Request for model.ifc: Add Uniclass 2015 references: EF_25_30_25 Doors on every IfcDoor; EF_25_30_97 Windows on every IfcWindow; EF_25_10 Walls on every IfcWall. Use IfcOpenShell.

First a look at what the model holds.

```python
import ifcopenshell

model = ifcopenshell.open("model.ifc")
print(model.schema)
print("classifications:", [c.Name for c in model.by_type("IfcClassification")])
for ifc_class in ("IfcDoor", "IfcRoof", "IfcStair", "IfcWall", "IfcWindow"):
    print(ifc_class, len(model.by_type(ifc_class)))
```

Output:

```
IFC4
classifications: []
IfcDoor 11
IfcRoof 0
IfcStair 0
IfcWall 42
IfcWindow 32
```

```python
import ifcopenshell
import ifcopenshell.api.classification

model = ifcopenshell.open("model.ifc")

system = ifcopenshell.api.classification.add_classification(model, classification="Uniclass 2015")

codes = {
    "IfcDoor": ("EF_25_30_25", "Doors"),
    "IfcWindow": ("EF_25_30_97", "Windows"),
    "IfcWall": ("EF_25_10", "Walls"),
}
for ifc_class, (code, name) in codes.items():
    products = model.by_type(ifc_class)
    ifcopenshell.api.classification.add_reference(
        model, products=products, classification=system, identification=code, name=name
    )
    print(code, len(products))

model.write("model_v2.ifc")
```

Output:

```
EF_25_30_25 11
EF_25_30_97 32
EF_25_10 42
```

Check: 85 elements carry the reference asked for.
